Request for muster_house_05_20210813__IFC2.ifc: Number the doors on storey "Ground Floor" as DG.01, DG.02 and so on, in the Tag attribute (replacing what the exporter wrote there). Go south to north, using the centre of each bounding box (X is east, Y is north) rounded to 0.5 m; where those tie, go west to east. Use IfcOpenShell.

First a look at what the model holds.

```python
import ifcopenshell
import ifcopenshell.util.element
import ifcopenshell.util.placement

model = ifcopenshell.open("muster_house_05_20210813__IFC2.ifc")
print(model.schema)
storey = next(s for s in model.by_type("IfcBuildingStorey") if s.Name == "Ground Floor")
doors = [e for e in ifcopenshell.util.element.get_decomposition(storey) if e.is_a("IfcDoor")]
for e in sorted(doors, key=lambda e: e.id()):
    origin = ifcopenshell.util.placement.get_local_placement(e.ObjectPlacement)[:3, 3]
    print(e.id(), e.Tag, e.Name, origin.round(2) + 0.0, sep=" | ")
```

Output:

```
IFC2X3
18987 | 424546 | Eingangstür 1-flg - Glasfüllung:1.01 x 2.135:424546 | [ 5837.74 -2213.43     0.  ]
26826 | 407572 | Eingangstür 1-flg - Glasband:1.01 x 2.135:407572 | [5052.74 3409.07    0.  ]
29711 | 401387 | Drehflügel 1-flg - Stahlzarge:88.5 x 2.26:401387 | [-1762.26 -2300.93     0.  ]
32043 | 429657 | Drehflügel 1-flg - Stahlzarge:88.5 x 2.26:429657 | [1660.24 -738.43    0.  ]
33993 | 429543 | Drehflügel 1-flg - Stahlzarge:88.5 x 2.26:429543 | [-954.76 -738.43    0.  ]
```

```python
import ifcopenshell
import ifcopenshell.geom
import ifcopenshell.util.element
import ifcopenshell.util.shape

model = ifcopenshell.open("muster_house_05_20210813__IFC2.ifc")
settings = ifcopenshell.geom.settings()
settings.set("use-world-coords", True)


def centre(element):
    shape = ifcopenshell.geom.create_shape(settings, element)
    return ifcopenshell.util.shape.get_bbox_centroid(shape.geometry)


storey = next(s for s in model.by_type("IfcBuildingStorey") if s.Name == "Ground Floor")
doors = [e for e in ifcopenshell.util.element.get_decomposition(storey) if e.is_a("IfcDoor")]

# Insertion points can sit at a corner or the storey origin, so sort by the geometry (in metres).
centres = {e: centre(e) for e in doors}
doors.sort(key=lambda e: (round(centres[e][1] / 0.5), centres[e][0]))

for i, e in enumerate(doors, start=1):
    number = f"DG.{i:02d}"
    e.Tag = number
    print(e.id(), number)

model.write("muster_house_05_20210813__IFC2_updated.ifc")
```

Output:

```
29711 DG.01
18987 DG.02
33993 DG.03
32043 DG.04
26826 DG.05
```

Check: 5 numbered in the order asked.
